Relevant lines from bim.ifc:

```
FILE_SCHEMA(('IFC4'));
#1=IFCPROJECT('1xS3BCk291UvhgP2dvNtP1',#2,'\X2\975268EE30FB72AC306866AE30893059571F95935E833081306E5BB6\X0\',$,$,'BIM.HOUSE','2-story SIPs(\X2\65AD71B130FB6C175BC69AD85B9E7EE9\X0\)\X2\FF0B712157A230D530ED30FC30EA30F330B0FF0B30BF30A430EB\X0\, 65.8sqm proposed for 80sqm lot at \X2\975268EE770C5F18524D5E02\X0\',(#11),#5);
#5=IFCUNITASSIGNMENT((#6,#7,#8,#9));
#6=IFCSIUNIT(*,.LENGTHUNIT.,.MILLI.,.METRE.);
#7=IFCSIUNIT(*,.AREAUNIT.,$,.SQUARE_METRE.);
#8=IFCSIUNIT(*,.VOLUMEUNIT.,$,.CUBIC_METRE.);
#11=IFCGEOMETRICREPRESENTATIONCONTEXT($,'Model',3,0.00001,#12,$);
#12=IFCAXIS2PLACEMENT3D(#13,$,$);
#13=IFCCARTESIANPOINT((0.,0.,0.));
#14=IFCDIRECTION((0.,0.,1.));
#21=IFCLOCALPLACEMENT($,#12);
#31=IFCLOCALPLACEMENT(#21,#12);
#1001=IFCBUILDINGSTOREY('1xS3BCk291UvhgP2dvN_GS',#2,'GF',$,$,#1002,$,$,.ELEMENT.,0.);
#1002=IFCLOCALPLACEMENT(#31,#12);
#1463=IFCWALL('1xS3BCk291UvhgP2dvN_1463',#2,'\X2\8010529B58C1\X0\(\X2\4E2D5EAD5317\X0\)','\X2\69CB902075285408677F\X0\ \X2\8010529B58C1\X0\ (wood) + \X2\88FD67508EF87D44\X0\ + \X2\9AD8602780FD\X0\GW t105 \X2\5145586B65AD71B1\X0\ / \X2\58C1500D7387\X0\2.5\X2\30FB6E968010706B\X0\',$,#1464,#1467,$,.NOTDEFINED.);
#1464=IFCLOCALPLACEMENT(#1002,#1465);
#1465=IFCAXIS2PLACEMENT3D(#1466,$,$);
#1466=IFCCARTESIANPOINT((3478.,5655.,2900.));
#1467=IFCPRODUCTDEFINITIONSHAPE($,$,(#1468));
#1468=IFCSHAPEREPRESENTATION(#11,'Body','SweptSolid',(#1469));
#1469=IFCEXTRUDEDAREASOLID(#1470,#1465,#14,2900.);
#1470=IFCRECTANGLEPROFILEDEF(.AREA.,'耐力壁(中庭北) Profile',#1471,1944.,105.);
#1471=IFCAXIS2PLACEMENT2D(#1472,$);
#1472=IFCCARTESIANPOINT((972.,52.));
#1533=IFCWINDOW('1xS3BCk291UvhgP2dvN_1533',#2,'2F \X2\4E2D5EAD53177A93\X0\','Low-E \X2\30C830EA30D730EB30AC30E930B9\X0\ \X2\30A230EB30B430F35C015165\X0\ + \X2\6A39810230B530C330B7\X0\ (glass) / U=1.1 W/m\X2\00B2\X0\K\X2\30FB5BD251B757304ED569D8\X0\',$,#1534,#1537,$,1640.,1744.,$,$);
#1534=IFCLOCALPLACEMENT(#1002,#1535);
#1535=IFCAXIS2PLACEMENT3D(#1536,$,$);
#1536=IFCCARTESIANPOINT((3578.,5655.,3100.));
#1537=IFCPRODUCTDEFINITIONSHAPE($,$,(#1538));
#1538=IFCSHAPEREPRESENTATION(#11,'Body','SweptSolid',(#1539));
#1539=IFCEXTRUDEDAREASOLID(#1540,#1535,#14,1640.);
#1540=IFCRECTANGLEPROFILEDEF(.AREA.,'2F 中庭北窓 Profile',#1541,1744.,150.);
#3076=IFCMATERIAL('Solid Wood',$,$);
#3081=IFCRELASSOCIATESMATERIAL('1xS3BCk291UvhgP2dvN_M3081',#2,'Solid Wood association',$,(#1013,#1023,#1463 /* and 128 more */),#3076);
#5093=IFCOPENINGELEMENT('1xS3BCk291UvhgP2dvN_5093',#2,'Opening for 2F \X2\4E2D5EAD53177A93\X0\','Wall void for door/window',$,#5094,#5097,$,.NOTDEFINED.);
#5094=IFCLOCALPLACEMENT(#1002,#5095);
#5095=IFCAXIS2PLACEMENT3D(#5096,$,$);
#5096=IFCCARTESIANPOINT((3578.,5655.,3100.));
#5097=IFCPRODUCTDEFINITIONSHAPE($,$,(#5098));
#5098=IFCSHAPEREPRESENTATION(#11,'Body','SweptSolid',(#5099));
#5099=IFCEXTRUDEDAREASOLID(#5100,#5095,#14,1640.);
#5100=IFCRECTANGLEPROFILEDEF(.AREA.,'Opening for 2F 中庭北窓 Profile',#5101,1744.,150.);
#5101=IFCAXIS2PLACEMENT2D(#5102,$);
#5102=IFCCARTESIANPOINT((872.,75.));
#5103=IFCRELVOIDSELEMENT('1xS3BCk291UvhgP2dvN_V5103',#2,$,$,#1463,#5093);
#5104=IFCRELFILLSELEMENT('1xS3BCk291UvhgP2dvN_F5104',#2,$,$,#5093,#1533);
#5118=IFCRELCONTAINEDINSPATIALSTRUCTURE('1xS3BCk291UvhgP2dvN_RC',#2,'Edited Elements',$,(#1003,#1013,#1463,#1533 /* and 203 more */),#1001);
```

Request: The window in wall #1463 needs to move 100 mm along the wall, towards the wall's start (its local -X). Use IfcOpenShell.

```python
import ifcopenshell
import ifcopenshell.api.geometry
import ifcopenshell.util.placement
import ifcopenshell.util.unit

model = ifcopenshell.open("bim.ifc")
unit_scale = ifcopenshell.util.unit.calculate_unit_scale(model)

window = model.by_guid("1xS3BCk291UvhgP2dvN_1533")
opening = window.FillsVoids[0].RelatingOpeningElement
wall = opening.VoidsElements[0].RelatingBuildingElement

wall_matrix = ifcopenshell.util.placement.get_local_placement(wall.ObjectPlacement)
shift = wall_matrix[:3, 0] * -0.1 / unit_scale
before = ifcopenshell.util.placement.get_local_placement(window.ObjectPlacement)[:3, 3].copy()

# The window is not placed relative to its opening, so move both.
for product in (opening, window):
    matrix = ifcopenshell.util.placement.get_local_placement(product.ObjectPlacement)
    matrix[:3, 3] += shift
    ifcopenshell.api.geometry.edit_object_placement(model, product=product, matrix=matrix, is_si=False)

after = ifcopenshell.util.placement.get_local_placement(window.ObjectPlacement)[:3, 3]
print("window moved by", (after - before).round(3) + 0.0)

model.write("bim_v2.ifc")
```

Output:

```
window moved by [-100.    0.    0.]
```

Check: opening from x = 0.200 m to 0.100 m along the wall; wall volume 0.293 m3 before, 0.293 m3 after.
